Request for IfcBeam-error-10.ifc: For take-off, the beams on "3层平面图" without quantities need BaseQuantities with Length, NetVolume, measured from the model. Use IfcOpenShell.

First a look at what the model holds.

```python
import ifcopenshell
import ifcopenshell.util.element
import ifcopenshell.util.unit

model = ifcopenshell.open("IfcBeam-error-10.ifc")
print(model.schema)
for unit_type in ("LENGTHUNIT", "AREAUNIT", "VOLUMEUNIT"):
    print(unit_type, ifcopenshell.util.unit.calculate_unit_scale(model, unit_type))
storey = next(s for s in model.by_type("IfcBuildingStorey") if s.Name == "3层平面图")
beams = [e for e in ifcopenshell.util.element.get_decomposition(storey) if e.is_a("IfcBeam")]
for e in sorted(beams, key=lambda e: e.id()):
    print(e.id(), e.is_a(), e.Name, list(ifcopenshell.util.element.get_psets(e, qtos_only=True)), sep=" | ")
```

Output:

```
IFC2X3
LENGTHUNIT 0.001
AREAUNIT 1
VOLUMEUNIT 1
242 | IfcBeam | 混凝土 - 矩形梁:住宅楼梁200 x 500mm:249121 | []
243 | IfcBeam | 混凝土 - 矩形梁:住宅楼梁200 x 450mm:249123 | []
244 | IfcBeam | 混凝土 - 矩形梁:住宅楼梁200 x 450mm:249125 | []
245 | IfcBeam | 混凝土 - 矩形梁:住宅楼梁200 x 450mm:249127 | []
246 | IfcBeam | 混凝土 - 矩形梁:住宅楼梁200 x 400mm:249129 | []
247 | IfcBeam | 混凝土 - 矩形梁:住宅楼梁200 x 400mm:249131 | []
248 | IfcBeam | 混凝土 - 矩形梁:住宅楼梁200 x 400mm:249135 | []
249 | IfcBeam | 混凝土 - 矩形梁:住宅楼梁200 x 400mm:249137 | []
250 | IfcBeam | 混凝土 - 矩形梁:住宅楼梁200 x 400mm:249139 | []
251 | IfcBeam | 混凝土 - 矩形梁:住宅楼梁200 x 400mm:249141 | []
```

```python
import ifcopenshell
import ifcopenshell.api.pset
import ifcopenshell.geom
import ifcopenshell.util.element
import ifcopenshell.util.shape
import ifcopenshell.util.unit

model = ifcopenshell.open("IfcBeam-error-10.ifc")
unit_scale = ifcopenshell.util.unit.calculate_unit_scale(model)
volume_scale = ifcopenshell.util.unit.calculate_unit_scale(model, "VOLUMEUNIT")
settings = ifcopenshell.geom.settings()

storey = next(s for s in model.by_type("IfcBuildingStorey") if s.Name == "3层平面图")
beams = [e for e in ifcopenshell.util.element.get_decomposition(storey) if e.is_a("IfcBeam")]

for e in sorted(beams, key=lambda e: e.id()):
    if ifcopenshell.util.element.get_psets(e, qtos_only=True, should_inherit=False):
        continue
    # Geometry comes back in metres, in the element's own axes.
    shape = ifcopenshell.geom.create_shape(settings, e)
    values = {
        "Length": ifcopenshell.util.shape.get_max_xyz(shape.geometry) / unit_scale,
        "NetVolume": ifcopenshell.util.shape.get_volume(shape.geometry) / volume_scale,
    }
    qto = ifcopenshell.api.pset.add_qto(model, product=e, name="BaseQuantities")
    ifcopenshell.api.pset.edit_qto(model, qto=qto, properties=values)
    print(e.id(), {k: round(v, 3) for k, v in values.items()})

model.write("IfcBeam-error-10_updated.ifc")
```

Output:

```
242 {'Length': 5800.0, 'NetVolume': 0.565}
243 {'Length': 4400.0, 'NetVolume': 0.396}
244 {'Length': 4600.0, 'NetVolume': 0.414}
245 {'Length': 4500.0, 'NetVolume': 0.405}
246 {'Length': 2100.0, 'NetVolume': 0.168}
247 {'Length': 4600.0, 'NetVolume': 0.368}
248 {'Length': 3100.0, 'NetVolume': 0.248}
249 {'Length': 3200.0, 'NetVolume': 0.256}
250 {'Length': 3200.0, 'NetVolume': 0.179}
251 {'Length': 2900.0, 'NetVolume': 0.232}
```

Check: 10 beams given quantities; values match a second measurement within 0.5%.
